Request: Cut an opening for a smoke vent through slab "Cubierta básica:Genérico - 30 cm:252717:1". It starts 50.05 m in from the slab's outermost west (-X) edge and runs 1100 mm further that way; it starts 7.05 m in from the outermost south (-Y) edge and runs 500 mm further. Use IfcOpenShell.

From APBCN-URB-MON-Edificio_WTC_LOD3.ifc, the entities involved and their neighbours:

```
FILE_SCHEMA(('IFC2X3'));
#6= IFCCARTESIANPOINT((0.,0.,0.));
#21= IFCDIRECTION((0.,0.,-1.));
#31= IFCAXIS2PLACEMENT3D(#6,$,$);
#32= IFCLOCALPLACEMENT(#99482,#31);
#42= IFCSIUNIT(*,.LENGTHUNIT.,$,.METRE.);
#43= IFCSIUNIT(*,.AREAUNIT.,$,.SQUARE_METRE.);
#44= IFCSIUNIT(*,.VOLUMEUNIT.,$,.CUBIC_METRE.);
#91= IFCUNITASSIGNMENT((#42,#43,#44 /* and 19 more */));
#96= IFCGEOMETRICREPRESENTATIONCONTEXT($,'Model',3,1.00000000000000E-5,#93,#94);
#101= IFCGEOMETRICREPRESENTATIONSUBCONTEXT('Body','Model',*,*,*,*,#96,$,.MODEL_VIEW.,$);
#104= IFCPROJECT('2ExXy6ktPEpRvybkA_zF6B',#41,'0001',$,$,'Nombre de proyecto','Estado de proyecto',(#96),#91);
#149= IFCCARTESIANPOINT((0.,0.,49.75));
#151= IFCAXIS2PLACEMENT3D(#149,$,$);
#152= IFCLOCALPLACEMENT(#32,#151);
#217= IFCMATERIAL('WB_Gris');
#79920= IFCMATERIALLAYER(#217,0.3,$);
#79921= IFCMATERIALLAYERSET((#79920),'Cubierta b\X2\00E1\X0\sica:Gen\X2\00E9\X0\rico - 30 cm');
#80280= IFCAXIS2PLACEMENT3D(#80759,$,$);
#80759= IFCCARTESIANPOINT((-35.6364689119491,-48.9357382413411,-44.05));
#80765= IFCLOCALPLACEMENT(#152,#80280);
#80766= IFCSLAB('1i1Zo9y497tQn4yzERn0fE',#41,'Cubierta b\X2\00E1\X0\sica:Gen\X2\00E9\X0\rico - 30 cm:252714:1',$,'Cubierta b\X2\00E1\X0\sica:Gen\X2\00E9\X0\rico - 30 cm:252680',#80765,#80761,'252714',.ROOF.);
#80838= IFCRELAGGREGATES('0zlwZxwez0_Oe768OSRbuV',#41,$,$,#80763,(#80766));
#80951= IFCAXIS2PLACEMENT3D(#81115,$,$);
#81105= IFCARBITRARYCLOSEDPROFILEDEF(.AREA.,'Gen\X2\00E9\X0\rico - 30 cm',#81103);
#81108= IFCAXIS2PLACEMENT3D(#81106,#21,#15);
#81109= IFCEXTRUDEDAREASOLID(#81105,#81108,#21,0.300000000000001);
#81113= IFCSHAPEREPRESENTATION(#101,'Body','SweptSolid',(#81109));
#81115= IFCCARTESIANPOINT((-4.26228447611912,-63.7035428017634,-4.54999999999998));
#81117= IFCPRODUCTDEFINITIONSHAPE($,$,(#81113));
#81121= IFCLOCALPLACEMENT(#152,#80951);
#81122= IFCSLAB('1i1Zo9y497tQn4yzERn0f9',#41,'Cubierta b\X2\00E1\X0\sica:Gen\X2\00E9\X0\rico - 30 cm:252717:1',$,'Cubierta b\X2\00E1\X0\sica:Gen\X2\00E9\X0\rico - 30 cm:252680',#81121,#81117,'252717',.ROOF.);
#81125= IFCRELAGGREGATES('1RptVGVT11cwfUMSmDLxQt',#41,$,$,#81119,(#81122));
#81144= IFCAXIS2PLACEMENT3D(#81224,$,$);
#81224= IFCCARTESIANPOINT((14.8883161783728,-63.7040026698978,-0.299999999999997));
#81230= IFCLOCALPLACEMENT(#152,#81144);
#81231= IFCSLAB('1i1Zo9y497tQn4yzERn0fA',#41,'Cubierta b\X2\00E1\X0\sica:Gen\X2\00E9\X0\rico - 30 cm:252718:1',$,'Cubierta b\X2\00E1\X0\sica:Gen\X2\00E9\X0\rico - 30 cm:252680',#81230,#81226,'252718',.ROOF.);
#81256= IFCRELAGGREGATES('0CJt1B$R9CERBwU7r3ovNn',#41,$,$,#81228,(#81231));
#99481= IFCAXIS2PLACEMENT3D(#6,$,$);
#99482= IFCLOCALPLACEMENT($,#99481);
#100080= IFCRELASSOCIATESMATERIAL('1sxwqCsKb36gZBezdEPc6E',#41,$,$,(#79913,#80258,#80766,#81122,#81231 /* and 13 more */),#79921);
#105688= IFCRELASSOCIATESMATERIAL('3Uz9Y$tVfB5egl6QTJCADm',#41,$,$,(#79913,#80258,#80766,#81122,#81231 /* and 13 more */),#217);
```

```python
import numpy as np
import ifcopenshell
import ifcopenshell.api.feature
import ifcopenshell.api.geometry
import ifcopenshell.api.root
import ifcopenshell.geom
import ifcopenshell.util.placement
import ifcopenshell.util.representation
import ifcopenshell.util.shape
import ifcopenshell.util.unit

model = ifcopenshell.open("APBCN-URB-MON-Edificio_WTC_LOD3.ifc")
unit_scale = ifcopenshell.util.unit.calculate_unit_scale(model)
settings = ifcopenshell.geom.settings()


def volume(element):
    """Net volume in cubic metres, openings subtracted."""
    shape = ifcopenshell.geom.create_shape(settings, element)
    return ifcopenshell.util.shape.get_volume(shape.geometry)


slab = model.by_guid("1i1Zo9y497tQn4yzERn0f9")
before = volume(slab)

# Extent in the slab's own axes, in metres. The edges named are its -X and -Y sides.
slab_shape = ifcopenshell.geom.create_shape(settings, slab)
vertices = ifcopenshell.util.shape.get_vertices(slab_shape.geometry)
x_min, y_min, bottom = vertices.min(axis=0)
top = vertices[:, 2].max()

opening = ifcopenshell.api.root.create_entity(model, ifc_class="IfcOpeningElement", name="Smoke vent opening")
context = ifcopenshell.util.representation.get_context(model, "Model", "Body", "MODEL_VIEW")
width, depth = 1.1, 0.5
outline = [(0.0, 0.0), (width, 0.0), (width, depth), (0.0, depth), (0.0, 0.0)]
# Overshoot both faces by 50 mm so the cut is clean.
shape = ifcopenshell.api.geometry.add_slab_representation(
    model, context=context, depth=top - bottom + 0.1, polyline=outline
)
ifcopenshell.api.geometry.assign_representation(model, product=opening, representation=shape)

matrix = ifcopenshell.util.placement.get_local_placement(slab.ObjectPlacement)
matrix[:, 3] = matrix @ np.append(np.array([x_min + 50.05, y_min + 7.05, bottom - 0.05]) / unit_scale, 1.0)
ifcopenshell.api.geometry.edit_object_placement(model, product=opening, matrix=matrix, is_si=False)
ifcopenshell.api.feature.add_feature(model, feature=opening, element=slab)

after = volume(slab)

print(f"slab volume {before:.3f} -> {after:.3f} m3")

model.write("APBCN-URB-MON-Edificio_WTC_LOD3-out.ifc")
```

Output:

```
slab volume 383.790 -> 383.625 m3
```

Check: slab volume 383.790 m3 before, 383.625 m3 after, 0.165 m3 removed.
